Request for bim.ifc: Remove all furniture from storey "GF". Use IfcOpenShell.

First a look at what the model holds.

```python
import ifcopenshell
import ifcopenshell.util.element

model = ifcopenshell.open("bim.ifc")
print(model.schema)
storey = next(s for s in model.by_type("IfcBuildingStorey") if s.Name == "GF")
furniture = [e for e in ifcopenshell.util.element.get_decomposition(storey) if e.is_a("IfcFurnishingElement")]
seen = {}
for e in furniture:
    element_type = ifcopenshell.util.element.get_type(e)
    name = element_type.Name if element_type not in (None, e) else None
    seen[name] = seen.get(name, 0) + 1
for name, count in sorted(seen.items(), key=str):
    print(count, "x", name)
```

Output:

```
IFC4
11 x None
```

```python
import ifcopenshell
import ifcopenshell.api.root
import ifcopenshell.util.element

model = ifcopenshell.open("bim.ifc")

storey = next(s for s in model.by_type("IfcBuildingStorey") if s.Name == "GF")
furniture = [e for e in ifcopenshell.util.element.get_decomposition(storey) if e.is_a("IfcFurnishingElement")]

for e in furniture:
    ifcopenshell.api.root.remove_product(model, product=e)
print(len(furniture), "removed")

model.write("bim_v2.ifc")
```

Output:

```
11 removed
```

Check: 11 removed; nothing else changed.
